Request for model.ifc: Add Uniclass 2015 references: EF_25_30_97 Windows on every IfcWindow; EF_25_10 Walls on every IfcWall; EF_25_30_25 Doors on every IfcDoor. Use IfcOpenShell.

First a look at what the model holds.

```python
import ifcopenshell

model = ifcopenshell.open("model.ifc")
print(model.schema)
print("classifications:", [c.Name for c in model.by_type("IfcClassification")])
for ifc_class in ("IfcDoor", "IfcRoof", "IfcStair", "IfcWall", "IfcWindow"):
    print(ifc_class, len(model.by_type(ifc_class)))
```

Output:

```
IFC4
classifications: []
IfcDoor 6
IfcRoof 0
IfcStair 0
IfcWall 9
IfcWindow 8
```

```python
import ifcopenshell
import ifcopenshell.api.classification

model = ifcopenshell.open("model.ifc")

system = ifcopenshell.api.classification.add_classification(model, classification="Uniclass 2015")

codes = {
    "IfcWindow": ("EF_25_30_97", "Windows"),
    "IfcWall": ("EF_25_10", "Walls"),
    "IfcDoor": ("EF_25_30_25", "Doors"),
}
for ifc_class, (code, name) in codes.items():
    products = model.by_type(ifc_class)
    ifcopenshell.api.classification.add_reference(
        model, products=products, classification=system, identification=code, name=name
    )
    print(code, len(products))

model.write("model_edited.ifc")
```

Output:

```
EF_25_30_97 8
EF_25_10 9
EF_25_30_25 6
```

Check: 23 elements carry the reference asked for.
